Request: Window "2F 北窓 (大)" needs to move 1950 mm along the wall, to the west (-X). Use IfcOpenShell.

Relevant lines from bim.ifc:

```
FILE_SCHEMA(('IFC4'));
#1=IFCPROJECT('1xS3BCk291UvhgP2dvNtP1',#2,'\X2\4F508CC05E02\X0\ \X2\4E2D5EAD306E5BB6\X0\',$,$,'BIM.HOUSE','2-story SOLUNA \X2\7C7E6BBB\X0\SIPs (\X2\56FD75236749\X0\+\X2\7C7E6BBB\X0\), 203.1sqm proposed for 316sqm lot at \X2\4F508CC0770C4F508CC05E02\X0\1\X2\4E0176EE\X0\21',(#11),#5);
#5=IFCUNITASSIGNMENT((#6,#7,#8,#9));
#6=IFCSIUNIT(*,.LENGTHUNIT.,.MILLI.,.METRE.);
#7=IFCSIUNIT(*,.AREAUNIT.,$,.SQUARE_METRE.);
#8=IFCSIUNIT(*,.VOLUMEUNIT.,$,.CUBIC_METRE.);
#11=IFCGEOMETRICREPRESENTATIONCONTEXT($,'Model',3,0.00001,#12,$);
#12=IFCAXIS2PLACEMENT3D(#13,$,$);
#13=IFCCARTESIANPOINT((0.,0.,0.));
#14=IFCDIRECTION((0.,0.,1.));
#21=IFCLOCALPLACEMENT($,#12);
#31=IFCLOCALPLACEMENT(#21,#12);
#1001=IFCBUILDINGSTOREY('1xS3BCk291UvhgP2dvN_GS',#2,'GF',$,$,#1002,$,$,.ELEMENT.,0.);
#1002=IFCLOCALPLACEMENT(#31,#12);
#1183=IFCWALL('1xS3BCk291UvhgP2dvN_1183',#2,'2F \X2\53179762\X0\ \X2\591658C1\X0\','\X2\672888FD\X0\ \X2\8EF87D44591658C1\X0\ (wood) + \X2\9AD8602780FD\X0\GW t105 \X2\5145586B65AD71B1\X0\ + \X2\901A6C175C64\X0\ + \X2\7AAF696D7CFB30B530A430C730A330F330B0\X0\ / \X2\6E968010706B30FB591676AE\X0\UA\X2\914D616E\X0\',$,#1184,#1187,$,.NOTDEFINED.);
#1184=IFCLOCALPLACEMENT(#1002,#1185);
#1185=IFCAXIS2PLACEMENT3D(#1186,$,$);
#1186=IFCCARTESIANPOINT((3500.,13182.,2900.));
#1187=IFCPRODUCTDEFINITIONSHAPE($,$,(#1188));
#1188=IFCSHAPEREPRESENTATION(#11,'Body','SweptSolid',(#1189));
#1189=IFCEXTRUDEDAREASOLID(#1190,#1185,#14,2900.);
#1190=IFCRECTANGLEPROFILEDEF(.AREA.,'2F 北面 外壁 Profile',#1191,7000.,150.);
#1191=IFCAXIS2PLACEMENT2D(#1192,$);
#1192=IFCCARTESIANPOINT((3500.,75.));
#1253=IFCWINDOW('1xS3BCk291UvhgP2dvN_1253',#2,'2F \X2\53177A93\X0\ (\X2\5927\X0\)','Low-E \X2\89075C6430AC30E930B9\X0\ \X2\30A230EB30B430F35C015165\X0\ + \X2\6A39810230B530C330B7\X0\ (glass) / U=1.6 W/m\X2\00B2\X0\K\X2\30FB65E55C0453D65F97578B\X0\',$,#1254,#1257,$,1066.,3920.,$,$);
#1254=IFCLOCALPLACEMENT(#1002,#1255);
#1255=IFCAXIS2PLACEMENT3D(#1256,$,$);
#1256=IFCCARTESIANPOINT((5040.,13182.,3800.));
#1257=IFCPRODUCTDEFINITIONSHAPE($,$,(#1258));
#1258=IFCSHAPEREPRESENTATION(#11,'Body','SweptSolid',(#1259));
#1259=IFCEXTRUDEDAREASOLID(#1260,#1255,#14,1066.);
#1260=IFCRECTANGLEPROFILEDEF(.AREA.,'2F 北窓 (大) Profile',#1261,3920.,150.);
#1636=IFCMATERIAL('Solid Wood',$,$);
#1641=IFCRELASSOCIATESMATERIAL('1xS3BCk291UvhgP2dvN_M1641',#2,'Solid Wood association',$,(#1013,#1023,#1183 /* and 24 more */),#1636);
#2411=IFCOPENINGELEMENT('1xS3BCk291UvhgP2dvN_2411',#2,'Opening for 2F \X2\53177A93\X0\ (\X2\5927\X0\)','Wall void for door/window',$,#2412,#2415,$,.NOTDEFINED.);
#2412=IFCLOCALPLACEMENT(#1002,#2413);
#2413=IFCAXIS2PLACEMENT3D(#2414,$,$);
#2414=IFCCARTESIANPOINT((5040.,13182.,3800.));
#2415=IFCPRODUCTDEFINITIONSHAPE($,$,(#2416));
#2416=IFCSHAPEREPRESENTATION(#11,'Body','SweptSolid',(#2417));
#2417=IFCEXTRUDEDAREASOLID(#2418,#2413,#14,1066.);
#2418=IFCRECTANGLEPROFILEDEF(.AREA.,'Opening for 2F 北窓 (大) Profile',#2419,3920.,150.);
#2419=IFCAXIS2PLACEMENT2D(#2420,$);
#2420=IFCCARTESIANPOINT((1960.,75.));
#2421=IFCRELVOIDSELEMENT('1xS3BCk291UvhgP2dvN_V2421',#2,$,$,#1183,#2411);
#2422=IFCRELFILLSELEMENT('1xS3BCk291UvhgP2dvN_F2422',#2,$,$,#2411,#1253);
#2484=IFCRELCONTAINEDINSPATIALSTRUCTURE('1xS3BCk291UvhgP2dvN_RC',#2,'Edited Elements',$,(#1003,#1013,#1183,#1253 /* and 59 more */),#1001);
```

```python
import ifcopenshell
import ifcopenshell.api.geometry
import ifcopenshell.util.placement

model = ifcopenshell.open("bim.ifc")

window = model.by_guid("1xS3BCk291UvhgP2dvN_1253")
opening = window.FillsVoids[0].RelatingOpeningElement
wall = opening.VoidsElements[0].RelatingBuildingElement

wall_matrix = ifcopenshell.util.placement.get_local_placement(wall.ObjectPlacement)
shift = wall_matrix[:3, 0] * -1950.0
before = ifcopenshell.util.placement.get_local_placement(window.ObjectPlacement)[:3, 3].copy()

# The window is not placed relative to its opening, so move both.
for product in (opening, window):
    matrix = ifcopenshell.util.placement.get_local_placement(product.ObjectPlacement)
    matrix[:3, 3] += shift
    ifcopenshell.api.geometry.edit_object_placement(model, product=product, matrix=matrix, is_si=False)

after = ifcopenshell.util.placement.get_local_placement(window.ObjectPlacement)[:3, 3]
print("window moved by", (after - before).round(3) + 0.0)

model.write("bim_rev.ifc")
```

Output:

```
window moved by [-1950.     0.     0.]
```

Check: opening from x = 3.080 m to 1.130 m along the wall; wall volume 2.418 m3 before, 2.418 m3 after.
